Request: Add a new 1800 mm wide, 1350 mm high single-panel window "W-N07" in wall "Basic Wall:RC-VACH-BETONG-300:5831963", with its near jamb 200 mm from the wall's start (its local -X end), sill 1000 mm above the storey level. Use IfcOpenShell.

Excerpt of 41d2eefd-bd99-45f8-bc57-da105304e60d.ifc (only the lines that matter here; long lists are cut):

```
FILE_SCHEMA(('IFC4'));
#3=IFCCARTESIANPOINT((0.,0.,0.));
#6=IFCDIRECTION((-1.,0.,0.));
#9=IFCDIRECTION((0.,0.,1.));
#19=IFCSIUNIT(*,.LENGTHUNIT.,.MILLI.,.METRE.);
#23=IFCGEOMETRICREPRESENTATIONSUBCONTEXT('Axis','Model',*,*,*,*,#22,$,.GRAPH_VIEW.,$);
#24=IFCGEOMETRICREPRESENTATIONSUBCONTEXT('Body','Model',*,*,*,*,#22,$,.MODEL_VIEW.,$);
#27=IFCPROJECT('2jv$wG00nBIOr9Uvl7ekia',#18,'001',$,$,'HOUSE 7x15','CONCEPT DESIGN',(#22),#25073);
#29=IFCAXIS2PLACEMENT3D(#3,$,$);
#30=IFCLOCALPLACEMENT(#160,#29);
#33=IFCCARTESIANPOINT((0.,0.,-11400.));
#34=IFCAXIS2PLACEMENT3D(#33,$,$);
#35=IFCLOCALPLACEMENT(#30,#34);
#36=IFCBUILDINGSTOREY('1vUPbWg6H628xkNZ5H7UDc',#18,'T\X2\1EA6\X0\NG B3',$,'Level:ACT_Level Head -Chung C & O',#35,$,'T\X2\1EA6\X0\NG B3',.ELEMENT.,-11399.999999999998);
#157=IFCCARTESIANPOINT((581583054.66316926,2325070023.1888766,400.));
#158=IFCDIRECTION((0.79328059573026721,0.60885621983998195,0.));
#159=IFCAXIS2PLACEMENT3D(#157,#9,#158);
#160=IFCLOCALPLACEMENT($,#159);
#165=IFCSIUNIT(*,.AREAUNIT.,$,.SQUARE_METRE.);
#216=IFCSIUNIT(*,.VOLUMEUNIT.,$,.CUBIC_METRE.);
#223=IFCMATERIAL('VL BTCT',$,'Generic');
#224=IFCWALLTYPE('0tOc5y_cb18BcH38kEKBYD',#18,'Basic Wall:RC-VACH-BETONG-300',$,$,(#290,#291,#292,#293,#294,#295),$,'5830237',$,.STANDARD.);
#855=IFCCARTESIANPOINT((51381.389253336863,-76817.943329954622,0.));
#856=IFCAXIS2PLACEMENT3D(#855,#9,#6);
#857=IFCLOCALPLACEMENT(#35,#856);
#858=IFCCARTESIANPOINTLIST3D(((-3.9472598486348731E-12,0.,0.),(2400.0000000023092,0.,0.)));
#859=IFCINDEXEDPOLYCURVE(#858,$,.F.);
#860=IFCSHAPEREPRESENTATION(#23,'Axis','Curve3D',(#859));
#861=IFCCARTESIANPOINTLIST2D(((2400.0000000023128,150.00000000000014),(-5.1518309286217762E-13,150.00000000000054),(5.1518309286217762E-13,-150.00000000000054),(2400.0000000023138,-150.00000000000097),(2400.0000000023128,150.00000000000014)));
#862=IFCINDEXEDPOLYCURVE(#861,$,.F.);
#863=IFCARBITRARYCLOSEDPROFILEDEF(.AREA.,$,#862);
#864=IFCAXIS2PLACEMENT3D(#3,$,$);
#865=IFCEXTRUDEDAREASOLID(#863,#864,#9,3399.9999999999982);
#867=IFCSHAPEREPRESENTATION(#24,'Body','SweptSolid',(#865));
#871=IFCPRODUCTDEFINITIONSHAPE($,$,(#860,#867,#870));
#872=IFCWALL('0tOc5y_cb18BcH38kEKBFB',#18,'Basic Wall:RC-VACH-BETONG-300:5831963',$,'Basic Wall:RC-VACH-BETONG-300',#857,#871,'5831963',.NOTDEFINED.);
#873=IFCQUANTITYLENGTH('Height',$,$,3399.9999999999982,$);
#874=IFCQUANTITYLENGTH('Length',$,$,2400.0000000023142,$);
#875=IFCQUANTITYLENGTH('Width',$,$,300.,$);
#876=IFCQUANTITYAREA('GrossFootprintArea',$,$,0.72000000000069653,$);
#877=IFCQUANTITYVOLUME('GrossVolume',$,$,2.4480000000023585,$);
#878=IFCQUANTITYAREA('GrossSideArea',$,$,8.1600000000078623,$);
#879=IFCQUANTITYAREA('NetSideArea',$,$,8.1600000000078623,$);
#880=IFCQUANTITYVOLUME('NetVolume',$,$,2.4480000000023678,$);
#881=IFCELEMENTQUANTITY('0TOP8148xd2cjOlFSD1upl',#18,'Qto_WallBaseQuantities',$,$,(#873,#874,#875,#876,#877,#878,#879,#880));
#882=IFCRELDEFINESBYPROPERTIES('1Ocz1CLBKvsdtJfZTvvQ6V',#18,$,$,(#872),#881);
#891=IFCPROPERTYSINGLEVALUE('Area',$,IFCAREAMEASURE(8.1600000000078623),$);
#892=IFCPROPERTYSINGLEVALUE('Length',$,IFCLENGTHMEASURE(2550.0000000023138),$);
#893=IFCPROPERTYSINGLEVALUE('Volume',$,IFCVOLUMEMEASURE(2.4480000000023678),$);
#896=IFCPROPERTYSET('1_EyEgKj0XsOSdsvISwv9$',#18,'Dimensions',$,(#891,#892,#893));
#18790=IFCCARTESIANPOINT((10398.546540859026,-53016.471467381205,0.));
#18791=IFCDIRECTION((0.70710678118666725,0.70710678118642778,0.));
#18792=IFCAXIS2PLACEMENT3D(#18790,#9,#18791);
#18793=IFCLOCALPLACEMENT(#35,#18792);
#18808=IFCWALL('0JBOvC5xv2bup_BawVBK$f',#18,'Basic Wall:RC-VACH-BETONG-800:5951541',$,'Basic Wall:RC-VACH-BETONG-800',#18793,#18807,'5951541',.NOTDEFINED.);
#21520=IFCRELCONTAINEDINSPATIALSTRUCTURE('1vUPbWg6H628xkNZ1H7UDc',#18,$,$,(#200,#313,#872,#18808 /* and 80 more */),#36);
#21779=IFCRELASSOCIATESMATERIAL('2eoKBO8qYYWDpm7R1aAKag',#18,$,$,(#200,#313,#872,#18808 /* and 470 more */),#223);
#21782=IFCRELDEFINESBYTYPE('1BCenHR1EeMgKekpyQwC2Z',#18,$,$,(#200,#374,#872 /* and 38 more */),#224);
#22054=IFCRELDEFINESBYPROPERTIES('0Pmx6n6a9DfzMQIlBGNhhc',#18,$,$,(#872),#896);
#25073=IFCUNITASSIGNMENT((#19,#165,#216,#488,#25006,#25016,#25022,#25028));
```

```python
import numpy as np
import ifcopenshell
import ifcopenshell.api.feature
import ifcopenshell.api.geometry
import ifcopenshell.api.pset
import ifcopenshell.api.root
import ifcopenshell.api.spatial
import ifcopenshell.geom
import ifcopenshell.util.element
import ifcopenshell.util.placement
import ifcopenshell.util.representation
import ifcopenshell.util.shape
import ifcopenshell.util.unit

model = ifcopenshell.open("41d2eefd-bd99-45f8-bc57-da105304e60d.ifc")
unit_scale = ifcopenshell.util.unit.calculate_unit_scale(model)
area_scale = ifcopenshell.util.unit.calculate_unit_scale(model, "AREAUNIT")
volume_scale = ifcopenshell.util.unit.calculate_unit_scale(model, "VOLUMEUNIT")
settings = ifcopenshell.geom.settings()


def volume(element):
    """Net volume in cubic metres, openings subtracted."""
    shape = ifcopenshell.geom.create_shape(settings, element)
    return ifcopenshell.util.shape.get_volume(shape.geometry)


wall = model.by_guid("0tOc5y_cb18BcH38kEKBFB")
storey = ifcopenshell.util.element.get_container(wall, ifc_class="IfcBuildingStorey")
context = ifcopenshell.util.representation.get_context(model, "Model", "Body", "MODEL_VIEW")
before = volume(wall)

width, height, from_end, sill = 1.8, 1.35, 0.2, 1  # metres

# The wall runs along its own X axis, and the end named is its -X end.
wall_shape = ifcopenshell.geom.create_shape(settings, wall)
x, y, z = ifcopenshell.util.shape.get_vertices(wall_shape.geometry).T
start = x.min() + from_end
face, thickness = float(y.min()), float(y.max() - y.min())
wall_matrix = ifcopenshell.util.placement.get_local_placement(wall.ObjectPlacement)
level = ifcopenshell.util.placement.get_local_placement(storey.ObjectPlacement)[2, 3]


def in_wall(x, y):
    """Placement at x, y metres in the wall's axes, at sill height."""
    matrix = wall_matrix.copy()
    matrix[:, 3] = wall_matrix @ np.array([x / unit_scale, y / unit_scale, 0.0, 1.0])
    matrix[2, 3] = level + sill / unit_scale
    return matrix


# Opening: a box that overshoots both wall faces by 50 mm.
opening = ifcopenshell.api.root.create_entity(model, ifc_class="IfcOpeningElement", predefined_type="OPENING")
box = ifcopenshell.api.geometry.add_wall_representation(
    model, context=context, length=width, height=height, thickness=thickness + 0.1
)
ifcopenshell.api.geometry.assign_representation(model, product=opening, representation=box)
ifcopenshell.api.geometry.edit_object_placement(model, product=opening, matrix=in_wall(start, face - 0.05), is_si=False)
ifcopenshell.api.feature.add_feature(model, feature=opening, element=wall)

window = ifcopenshell.api.root.create_entity(model, ifc_class="IfcWindow", name="W-N07", predefined_type="WINDOW")
window.OverallWidth, window.OverallHeight = width / unit_scale, height / unit_scale
window.PartitioningType = "SINGLE_PANEL"
body = ifcopenshell.api.geometry.add_window_representation(
    model,
    context=context,
    overall_width=window.OverallWidth,
    overall_height=window.OverallHeight,
    partition_type="SINGLE_PANEL",
)
ifcopenshell.api.geometry.assign_representation(model, product=window, representation=body)
ifcopenshell.api.spatial.assign_container(model, products=[window], relating_structure=storey)
ifcopenshell.api.feature.add_filling(model, opening=opening, element=window)

# Centre the window in the wall's thickness.
ifcopenshell.api.geometry.edit_object_placement(model, product=window, matrix=in_wall(start, face), is_si=False)
window_shape = ifcopenshell.geom.create_shape(settings, window)
depth = ifcopenshell.util.shape.get_vertices(window_shape.geometry)[:, 1]
offset = face + thickness / 2 - (depth.min() + depth.max()) / 2
ifcopenshell.api.geometry.edit_object_placement(model, product=window, matrix=in_wall(start, offset), is_si=False)

after = volume(wall)

# Update the wall's stored quantities.
qto = model.by_id(ifcopenshell.util.element.get_pset(wall, "Qto_WallBaseQuantities", should_inherit=False)["id"])
ifcopenshell.api.pset.edit_qto(model, qto=qto, properties={
    "NetSideArea": after / thickness / area_scale,
    "NetVolume": after / volume_scale,
})
pset = model.by_id(ifcopenshell.util.element.get_pset(wall, "Dimensions", should_inherit=False)["id"])
ifcopenshell.api.pset.edit_pset(model, pset=pset, properties={
    "Area": model.create_entity("IfcAreaMeasure", after / thickness / area_scale),
    "Volume": model.create_entity("IfcVolumeMeasure", after / volume_scale),
})

print(f"wall volume {before:.3f} -> {after:.3f} m3")

model.write("41d2eefd-bd99-45f8-bc57-da105304e60d_rev.ifc")
```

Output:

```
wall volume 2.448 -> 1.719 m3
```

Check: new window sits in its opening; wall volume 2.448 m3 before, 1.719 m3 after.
